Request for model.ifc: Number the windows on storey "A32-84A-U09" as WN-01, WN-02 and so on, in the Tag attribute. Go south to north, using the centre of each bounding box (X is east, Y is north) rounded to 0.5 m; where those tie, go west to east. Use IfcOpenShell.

First a look at what the model holds.

```python
import ifcopenshell
import ifcopenshell.util.element
import ifcopenshell.util.placement

model = ifcopenshell.open("model.ifc")
print(model.schema)
storey = next(s for s in model.by_type("IfcBuildingStorey") if s.Name == "A32-84A-U09")
windows = [e for e in ifcopenshell.util.element.get_decomposition(storey) if e.is_a("IfcWindow")]
for e in sorted(windows, key=lambda e: e.id()):
    origin = ifcopenshell.util.placement.get_local_placement(e.ObjectPlacement)[:3, 3]
    print(e.id(), e.Tag, e.Name, origin.round(2) + 0.0, sep=" | ")
```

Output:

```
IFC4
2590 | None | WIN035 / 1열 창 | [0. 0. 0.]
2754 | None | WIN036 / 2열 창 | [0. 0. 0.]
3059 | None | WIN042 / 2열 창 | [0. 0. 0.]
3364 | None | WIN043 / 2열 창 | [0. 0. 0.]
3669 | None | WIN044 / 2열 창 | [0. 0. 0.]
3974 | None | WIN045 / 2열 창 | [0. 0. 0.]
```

```python
import ifcopenshell
import ifcopenshell.geom
import ifcopenshell.util.element
import ifcopenshell.util.shape

model = ifcopenshell.open("model.ifc")
settings = ifcopenshell.geom.settings()
settings.set("use-world-coords", True)


def centre(element):
    shape = ifcopenshell.geom.create_shape(settings, element)
    return ifcopenshell.util.shape.get_bbox_centroid(shape.geometry)


storey = next(s for s in model.by_type("IfcBuildingStorey") if s.Name == "A32-84A-U09")
windows = [e for e in ifcopenshell.util.element.get_decomposition(storey) if e.is_a("IfcWindow")]

# Insertion points can sit at a corner or the storey origin, so sort by the geometry (in metres).
centres = {e: centre(e) for e in windows}
windows.sort(key=lambda e: (round(centres[e][1] / 0.5), centres[e][0]))

for i, e in enumerate(windows, start=1):
    number = f"WN-{i:02d}"
    e.Tag = number
    print(e.id(), number)

model.write("model_edited.ifc")
```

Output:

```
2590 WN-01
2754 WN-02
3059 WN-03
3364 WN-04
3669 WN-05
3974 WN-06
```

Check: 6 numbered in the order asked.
